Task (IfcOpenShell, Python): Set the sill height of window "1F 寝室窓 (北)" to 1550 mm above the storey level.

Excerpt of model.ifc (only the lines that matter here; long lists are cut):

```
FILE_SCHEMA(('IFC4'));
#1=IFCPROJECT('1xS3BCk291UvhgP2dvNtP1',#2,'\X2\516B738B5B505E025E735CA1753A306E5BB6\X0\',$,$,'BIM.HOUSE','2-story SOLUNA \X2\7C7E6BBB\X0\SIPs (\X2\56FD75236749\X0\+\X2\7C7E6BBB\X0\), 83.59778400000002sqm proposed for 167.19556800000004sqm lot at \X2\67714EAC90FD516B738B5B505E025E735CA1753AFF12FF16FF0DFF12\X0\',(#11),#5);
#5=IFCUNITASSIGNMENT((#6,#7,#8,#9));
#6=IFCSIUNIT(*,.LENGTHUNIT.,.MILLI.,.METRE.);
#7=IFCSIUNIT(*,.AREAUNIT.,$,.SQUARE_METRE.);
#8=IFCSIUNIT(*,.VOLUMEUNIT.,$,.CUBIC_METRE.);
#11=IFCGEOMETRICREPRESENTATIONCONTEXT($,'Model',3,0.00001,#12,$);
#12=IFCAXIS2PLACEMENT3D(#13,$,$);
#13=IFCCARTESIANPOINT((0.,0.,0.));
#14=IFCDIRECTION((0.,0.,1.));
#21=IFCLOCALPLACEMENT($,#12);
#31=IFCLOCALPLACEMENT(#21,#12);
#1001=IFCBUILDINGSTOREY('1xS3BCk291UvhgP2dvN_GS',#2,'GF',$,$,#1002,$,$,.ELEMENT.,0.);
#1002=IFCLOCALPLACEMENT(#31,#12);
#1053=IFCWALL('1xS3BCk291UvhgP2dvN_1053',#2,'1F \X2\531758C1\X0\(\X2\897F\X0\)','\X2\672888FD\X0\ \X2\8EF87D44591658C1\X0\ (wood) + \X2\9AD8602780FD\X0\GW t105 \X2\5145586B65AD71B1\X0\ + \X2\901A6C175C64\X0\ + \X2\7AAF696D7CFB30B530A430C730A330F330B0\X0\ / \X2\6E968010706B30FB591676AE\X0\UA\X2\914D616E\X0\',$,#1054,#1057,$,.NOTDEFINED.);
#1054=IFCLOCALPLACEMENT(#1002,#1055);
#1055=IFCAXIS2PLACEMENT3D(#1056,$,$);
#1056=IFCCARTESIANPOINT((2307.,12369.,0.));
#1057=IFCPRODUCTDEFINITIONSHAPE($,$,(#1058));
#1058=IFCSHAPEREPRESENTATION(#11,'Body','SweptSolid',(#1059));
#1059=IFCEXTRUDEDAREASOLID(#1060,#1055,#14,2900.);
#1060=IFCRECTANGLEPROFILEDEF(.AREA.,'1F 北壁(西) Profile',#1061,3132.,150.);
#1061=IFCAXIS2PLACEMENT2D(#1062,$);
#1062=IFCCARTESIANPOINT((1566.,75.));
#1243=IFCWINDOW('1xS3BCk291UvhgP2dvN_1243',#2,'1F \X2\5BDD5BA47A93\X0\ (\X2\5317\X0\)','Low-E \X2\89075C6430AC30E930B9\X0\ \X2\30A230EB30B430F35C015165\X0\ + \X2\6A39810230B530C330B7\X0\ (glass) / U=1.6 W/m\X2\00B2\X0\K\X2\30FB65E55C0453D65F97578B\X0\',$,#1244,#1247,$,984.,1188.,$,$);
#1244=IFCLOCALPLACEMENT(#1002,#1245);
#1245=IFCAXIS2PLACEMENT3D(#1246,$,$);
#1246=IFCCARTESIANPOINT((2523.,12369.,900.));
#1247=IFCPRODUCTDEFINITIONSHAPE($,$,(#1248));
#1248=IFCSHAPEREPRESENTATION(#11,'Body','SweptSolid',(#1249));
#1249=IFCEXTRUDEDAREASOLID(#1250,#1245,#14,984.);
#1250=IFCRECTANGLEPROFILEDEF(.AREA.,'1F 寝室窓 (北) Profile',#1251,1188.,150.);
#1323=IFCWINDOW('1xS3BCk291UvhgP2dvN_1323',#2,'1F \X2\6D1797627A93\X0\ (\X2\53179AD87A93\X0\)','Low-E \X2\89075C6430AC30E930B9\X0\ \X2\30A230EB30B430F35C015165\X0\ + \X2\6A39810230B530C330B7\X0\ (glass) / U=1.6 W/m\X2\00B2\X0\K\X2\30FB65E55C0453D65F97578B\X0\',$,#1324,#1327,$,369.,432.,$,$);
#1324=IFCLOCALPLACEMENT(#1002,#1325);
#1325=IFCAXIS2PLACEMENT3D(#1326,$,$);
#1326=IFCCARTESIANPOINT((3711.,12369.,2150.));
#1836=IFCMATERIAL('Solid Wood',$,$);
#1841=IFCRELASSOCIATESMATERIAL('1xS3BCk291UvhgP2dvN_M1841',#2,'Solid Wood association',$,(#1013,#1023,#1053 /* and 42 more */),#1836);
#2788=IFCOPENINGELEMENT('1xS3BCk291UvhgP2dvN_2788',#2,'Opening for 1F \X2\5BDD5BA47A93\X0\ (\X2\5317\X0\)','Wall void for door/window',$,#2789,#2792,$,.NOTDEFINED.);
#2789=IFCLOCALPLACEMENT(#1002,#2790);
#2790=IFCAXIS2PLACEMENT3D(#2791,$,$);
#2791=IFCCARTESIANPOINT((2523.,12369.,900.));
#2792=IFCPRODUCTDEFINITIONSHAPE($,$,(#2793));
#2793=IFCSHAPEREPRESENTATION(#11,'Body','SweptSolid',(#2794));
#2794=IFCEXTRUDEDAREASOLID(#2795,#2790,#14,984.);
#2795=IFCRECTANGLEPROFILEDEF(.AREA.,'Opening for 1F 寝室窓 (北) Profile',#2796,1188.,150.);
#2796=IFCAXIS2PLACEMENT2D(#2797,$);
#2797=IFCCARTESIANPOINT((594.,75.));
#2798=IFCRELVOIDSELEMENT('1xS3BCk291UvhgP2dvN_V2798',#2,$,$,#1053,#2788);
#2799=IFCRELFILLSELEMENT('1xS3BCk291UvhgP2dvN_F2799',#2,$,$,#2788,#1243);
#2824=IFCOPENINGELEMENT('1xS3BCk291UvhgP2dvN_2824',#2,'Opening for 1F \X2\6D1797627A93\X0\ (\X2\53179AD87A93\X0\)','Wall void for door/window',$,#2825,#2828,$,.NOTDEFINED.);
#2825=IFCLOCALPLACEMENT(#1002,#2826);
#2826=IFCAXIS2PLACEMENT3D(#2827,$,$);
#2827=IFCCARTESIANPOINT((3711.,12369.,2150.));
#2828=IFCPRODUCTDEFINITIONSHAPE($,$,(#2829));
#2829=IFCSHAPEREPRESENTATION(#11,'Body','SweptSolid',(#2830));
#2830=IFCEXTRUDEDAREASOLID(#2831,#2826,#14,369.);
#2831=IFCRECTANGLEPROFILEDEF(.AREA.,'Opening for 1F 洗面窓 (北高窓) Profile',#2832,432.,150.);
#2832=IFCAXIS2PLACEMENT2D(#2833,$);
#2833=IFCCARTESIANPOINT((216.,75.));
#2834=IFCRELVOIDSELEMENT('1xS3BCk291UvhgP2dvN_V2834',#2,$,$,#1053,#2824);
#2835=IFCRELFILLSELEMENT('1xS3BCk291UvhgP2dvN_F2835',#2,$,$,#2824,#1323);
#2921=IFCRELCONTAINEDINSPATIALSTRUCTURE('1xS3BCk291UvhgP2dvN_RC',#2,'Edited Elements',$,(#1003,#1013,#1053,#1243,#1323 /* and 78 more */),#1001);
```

```python
import numpy as np
import ifcopenshell
import ifcopenshell.api.geometry
import ifcopenshell.geom
import ifcopenshell.util.element
import ifcopenshell.util.placement
import ifcopenshell.util.shape
import ifcopenshell.util.unit

model = ifcopenshell.open("model.ifc")
unit_scale = ifcopenshell.util.unit.calculate_unit_scale(model)

window = model.by_guid("1xS3BCk291UvhgP2dvN_1243")
opening = window.FillsVoids[0].RelatingOpeningElement
storey = ifcopenshell.util.element.get_container(window, ifc_class="IfcBuildingStorey")
level = ifcopenshell.util.placement.get_local_placement(storey.ObjectPlacement)[2, 3]

# The opening's origin need not be at the sill, so measure its lowest point.
shape = ifcopenshell.geom.create_shape(ifcopenshell.geom.settings(), opening)
bottom = ifcopenshell.util.shape.get_shape_bottom_elevation(shape, shape.geometry) / unit_scale
dz = level + 1550.0 - bottom

shift = np.array([0.0, 0.0, dz])
# The window is not placed relative to its opening, so move both.
for product in (opening, window):
    matrix = ifcopenshell.util.placement.get_local_placement(product.ObjectPlacement)
    matrix[:3, 3] += shift
    ifcopenshell.api.geometry.edit_object_placement(model, product=product, matrix=matrix, is_si=False)

print(f"moved by {dz * unit_scale:+.3f} m")

model.write("model_v2.ifc")
```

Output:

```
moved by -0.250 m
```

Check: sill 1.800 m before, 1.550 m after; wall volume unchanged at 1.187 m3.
